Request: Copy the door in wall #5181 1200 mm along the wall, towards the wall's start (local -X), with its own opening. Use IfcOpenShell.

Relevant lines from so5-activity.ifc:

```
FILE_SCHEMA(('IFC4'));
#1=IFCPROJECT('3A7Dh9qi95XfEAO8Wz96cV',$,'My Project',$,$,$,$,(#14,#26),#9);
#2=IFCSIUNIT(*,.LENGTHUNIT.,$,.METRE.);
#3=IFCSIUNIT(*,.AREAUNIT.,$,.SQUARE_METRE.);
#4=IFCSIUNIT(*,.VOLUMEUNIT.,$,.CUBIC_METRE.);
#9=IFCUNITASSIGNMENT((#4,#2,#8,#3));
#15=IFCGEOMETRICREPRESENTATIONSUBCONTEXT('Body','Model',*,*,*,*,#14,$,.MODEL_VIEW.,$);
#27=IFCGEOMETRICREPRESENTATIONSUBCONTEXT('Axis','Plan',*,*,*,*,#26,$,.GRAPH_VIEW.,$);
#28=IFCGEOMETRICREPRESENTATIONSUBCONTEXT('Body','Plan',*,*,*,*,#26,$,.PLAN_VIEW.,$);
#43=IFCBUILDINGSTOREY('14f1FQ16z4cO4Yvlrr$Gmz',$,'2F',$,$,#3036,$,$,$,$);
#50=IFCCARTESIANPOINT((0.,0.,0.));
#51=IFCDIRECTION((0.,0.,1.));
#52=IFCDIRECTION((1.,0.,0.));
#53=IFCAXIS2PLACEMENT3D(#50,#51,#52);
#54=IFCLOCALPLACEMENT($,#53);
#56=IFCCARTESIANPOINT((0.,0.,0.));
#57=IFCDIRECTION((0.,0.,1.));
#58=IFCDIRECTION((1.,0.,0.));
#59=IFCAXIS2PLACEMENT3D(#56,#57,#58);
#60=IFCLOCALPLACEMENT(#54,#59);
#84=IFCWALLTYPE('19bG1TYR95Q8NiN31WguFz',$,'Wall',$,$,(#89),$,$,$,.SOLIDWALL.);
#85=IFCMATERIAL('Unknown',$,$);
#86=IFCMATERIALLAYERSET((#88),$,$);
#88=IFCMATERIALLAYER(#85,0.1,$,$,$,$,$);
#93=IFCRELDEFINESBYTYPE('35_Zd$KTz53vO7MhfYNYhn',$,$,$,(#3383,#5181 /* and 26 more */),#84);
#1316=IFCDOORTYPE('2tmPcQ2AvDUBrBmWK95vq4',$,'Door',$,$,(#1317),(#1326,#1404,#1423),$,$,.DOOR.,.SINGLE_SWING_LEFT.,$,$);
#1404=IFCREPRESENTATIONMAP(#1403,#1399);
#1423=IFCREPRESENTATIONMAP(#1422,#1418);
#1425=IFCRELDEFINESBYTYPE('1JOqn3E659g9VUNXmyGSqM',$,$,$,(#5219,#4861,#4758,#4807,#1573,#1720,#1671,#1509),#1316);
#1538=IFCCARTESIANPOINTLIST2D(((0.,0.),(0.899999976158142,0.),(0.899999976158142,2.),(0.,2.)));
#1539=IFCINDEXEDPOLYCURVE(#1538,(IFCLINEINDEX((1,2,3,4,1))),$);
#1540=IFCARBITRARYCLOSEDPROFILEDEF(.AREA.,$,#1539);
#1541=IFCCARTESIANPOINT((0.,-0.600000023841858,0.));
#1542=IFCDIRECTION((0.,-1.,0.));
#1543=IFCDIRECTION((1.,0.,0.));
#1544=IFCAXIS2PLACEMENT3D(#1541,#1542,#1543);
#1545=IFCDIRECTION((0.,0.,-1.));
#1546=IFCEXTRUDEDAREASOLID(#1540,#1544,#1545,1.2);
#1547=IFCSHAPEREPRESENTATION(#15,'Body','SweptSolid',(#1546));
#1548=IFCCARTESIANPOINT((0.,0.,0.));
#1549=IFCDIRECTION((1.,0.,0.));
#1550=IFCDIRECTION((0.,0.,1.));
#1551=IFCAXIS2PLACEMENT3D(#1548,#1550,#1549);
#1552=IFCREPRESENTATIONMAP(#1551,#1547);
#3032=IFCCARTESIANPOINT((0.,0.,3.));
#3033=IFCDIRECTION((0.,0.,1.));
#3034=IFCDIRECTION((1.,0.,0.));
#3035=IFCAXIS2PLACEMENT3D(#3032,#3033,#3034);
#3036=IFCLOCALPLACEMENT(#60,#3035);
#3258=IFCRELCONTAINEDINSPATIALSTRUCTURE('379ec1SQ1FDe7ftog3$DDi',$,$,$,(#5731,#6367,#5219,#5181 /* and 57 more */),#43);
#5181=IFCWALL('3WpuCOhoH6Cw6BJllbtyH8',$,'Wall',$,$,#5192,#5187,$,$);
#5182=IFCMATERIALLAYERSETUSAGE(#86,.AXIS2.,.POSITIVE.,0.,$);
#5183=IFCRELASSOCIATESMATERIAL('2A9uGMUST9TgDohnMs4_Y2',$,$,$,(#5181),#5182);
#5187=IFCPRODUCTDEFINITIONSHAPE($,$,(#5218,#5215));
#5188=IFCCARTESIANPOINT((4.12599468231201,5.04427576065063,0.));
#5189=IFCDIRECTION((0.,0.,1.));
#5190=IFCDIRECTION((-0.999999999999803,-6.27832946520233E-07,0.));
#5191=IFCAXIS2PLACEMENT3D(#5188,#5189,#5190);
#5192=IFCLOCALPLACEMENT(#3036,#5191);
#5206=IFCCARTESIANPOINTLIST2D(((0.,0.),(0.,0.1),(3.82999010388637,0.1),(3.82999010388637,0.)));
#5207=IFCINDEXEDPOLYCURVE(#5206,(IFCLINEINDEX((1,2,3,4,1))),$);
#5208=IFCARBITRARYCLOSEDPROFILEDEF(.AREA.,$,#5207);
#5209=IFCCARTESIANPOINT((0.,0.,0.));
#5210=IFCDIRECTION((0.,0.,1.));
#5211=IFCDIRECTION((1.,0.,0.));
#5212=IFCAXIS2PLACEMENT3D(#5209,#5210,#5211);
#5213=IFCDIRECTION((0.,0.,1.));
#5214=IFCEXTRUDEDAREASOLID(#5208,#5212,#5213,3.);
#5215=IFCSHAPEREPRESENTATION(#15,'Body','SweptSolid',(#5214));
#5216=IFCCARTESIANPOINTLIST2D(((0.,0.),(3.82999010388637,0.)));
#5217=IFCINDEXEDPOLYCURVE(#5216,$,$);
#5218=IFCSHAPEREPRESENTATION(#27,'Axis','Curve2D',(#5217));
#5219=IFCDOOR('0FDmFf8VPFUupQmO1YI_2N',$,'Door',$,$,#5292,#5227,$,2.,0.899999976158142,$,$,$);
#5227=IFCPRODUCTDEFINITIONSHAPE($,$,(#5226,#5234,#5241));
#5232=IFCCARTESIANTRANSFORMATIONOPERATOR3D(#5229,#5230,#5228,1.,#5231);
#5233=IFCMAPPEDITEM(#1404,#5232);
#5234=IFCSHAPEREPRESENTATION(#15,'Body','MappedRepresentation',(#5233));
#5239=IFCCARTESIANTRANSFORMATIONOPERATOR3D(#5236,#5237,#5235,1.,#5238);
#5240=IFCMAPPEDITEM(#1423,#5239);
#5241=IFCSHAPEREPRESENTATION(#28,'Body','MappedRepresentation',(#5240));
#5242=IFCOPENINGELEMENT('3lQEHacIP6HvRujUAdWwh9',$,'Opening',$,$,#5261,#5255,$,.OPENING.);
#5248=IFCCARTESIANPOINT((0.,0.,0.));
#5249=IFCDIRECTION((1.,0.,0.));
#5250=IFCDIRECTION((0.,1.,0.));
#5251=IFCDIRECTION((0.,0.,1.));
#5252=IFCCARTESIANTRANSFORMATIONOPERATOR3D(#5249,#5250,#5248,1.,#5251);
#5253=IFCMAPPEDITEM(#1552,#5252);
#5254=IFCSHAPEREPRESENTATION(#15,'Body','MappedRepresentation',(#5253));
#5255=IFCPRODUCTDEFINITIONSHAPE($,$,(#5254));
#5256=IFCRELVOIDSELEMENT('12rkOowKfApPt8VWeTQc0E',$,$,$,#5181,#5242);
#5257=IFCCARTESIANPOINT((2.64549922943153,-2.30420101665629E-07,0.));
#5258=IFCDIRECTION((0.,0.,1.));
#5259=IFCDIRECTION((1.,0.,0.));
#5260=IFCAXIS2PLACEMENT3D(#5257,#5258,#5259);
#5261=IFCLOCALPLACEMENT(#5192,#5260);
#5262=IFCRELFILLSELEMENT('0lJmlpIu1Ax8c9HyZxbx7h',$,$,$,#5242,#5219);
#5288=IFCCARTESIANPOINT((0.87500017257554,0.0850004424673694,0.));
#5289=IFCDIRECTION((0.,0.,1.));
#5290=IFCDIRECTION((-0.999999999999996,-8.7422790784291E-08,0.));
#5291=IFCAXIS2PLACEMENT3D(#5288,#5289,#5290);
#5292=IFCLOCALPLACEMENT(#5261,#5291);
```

```python
import ifcopenshell
import ifcopenshell.api.feature
import ifcopenshell.api.geometry
import ifcopenshell.api.root
import ifcopenshell.geom
import ifcopenshell.util.element
import ifcopenshell.util.placement
import ifcopenshell.util.shape

model = ifcopenshell.open("so5-activity.ifc")
settings = ifcopenshell.geom.settings()


def volume(element):
    """Net volume in cubic metres, openings subtracted."""
    shape = ifcopenshell.geom.create_shape(settings, element)
    return ifcopenshell.util.shape.get_volume(shape.geometry)


door = model.by_id(5219)
opening = door.FillsVoids[0].RelatingOpeningElement
wall = opening.VoidsElements[0].RelatingBuildingElement
before = volume(wall)
shift = ifcopenshell.util.placement.get_local_placement(wall.ObjectPlacement)[:3, 0] * -1.2

# copy_class copies the void relationship, type, container and properties, but no geometry.
new_opening = ifcopenshell.api.root.copy_class(model, product=opening)
new_opening.Representation = ifcopenshell.util.element.copy_deep(
    model, opening.Representation, exclude=["IfcGeometricRepresentationContext", "IfcRepresentationMap"]
)
new_door = ifcopenshell.api.root.copy_class(model, product=door)
new_door.Representation = ifcopenshell.util.element.copy_deep(
    model, door.Representation, exclude=["IfcGeometricRepresentationContext", "IfcRepresentationMap"]
)
ifcopenshell.api.feature.add_filling(model, opening=new_opening, element=new_door)

for old, new in ((opening, new_opening), (door, new_door)):
    matrix = ifcopenshell.util.placement.get_local_placement(old.ObjectPlacement)
    matrix[:3, 3] += shift
    ifcopenshell.api.geometry.edit_object_placement(model, product=new, matrix=matrix, is_si=False)

after = volume(wall)

print(f"wall volume {before:.3f} -> {after:.3f} m3")

model.write("so5-activity_edited.ifc")
```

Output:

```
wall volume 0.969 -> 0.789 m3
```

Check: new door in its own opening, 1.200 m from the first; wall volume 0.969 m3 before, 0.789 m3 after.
